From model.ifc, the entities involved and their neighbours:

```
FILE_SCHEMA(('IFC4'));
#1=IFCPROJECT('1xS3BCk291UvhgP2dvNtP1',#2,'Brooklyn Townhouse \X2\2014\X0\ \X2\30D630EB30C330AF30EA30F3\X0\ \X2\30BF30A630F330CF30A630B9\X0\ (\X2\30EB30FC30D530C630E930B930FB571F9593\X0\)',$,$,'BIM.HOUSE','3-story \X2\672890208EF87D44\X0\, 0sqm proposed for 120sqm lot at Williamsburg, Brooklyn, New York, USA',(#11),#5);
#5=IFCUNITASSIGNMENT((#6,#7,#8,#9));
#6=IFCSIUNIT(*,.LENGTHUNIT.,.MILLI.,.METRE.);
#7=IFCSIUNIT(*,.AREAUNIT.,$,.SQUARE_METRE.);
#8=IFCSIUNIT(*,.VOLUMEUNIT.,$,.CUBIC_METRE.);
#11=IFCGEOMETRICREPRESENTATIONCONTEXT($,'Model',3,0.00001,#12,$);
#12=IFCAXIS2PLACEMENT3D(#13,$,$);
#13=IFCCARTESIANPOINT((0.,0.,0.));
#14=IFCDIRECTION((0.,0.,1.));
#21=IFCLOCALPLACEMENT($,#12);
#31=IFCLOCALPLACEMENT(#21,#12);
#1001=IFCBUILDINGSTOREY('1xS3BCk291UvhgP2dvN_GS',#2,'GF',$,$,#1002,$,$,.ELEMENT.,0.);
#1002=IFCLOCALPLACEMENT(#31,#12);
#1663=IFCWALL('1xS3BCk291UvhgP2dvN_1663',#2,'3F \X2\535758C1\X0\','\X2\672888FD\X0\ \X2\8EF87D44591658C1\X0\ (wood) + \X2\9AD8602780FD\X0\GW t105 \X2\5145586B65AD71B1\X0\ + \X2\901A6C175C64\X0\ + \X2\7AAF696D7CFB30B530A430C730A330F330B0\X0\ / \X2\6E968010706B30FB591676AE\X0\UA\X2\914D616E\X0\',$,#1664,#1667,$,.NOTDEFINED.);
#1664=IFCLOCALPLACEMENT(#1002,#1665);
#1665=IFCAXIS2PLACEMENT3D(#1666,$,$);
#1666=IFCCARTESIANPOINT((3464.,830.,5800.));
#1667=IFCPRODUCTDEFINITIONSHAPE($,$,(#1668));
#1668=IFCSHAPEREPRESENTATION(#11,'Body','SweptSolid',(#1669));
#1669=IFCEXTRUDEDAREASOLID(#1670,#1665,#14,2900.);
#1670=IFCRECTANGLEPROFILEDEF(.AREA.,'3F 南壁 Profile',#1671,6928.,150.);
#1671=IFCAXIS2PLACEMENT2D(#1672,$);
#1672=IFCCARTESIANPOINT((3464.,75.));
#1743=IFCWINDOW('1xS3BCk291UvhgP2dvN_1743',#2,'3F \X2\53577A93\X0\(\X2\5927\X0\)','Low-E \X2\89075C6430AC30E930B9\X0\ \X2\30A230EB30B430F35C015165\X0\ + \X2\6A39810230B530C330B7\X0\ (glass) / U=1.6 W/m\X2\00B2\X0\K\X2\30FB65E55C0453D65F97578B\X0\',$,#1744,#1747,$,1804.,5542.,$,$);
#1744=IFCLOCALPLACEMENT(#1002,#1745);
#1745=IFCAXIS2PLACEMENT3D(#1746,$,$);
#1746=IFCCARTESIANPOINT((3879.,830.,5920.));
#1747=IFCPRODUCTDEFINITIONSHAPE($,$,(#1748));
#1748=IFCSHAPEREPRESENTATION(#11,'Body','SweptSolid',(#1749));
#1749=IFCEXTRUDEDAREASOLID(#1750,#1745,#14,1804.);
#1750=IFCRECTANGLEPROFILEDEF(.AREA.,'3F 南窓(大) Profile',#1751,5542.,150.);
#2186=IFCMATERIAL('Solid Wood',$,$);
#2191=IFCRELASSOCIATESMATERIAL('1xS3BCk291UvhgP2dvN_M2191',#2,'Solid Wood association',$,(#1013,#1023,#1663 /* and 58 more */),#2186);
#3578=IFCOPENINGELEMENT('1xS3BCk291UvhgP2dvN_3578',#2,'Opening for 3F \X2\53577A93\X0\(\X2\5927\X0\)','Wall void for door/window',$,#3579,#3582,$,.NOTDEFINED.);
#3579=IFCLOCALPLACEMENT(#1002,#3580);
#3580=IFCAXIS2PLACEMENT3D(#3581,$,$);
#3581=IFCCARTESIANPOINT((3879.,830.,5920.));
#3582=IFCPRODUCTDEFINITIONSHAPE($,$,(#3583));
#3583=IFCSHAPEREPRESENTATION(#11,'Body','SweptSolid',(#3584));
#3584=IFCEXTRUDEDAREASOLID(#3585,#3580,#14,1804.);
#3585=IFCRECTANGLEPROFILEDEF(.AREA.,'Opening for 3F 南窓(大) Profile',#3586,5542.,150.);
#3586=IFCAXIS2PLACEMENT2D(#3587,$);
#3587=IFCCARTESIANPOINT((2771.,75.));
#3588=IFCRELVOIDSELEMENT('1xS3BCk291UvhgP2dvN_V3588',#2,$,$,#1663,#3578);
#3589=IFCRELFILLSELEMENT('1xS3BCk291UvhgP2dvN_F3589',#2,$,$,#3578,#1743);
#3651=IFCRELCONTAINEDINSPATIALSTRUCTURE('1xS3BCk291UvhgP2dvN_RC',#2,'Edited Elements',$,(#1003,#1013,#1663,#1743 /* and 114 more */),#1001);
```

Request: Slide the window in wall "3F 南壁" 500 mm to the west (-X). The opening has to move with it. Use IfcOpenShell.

```python
import ifcopenshell
import ifcopenshell.api.geometry
import ifcopenshell.util.placement
import ifcopenshell.util.unit

model = ifcopenshell.open("model.ifc")
unit_scale = ifcopenshell.util.unit.calculate_unit_scale(model)

window = model.by_id(1743)
opening = window.FillsVoids[0].RelatingOpeningElement
wall = opening.VoidsElements[0].RelatingBuildingElement

wall_matrix = ifcopenshell.util.placement.get_local_placement(wall.ObjectPlacement)
shift = wall_matrix[:3, 0] * -0.5 / unit_scale
before = ifcopenshell.util.placement.get_local_placement(window.ObjectPlacement)[:3, 3].copy()

# The window is not placed relative to its opening, so move both.
for product in (opening, window):
    matrix = ifcopenshell.util.placement.get_local_placement(product.ObjectPlacement)
    matrix[:3, 3] += shift
    ifcopenshell.api.geometry.edit_object_placement(model, product=product, matrix=matrix, is_si=False)

after = ifcopenshell.util.placement.get_local_placement(window.ObjectPlacement)[:3, 3]
print("window moved by", (after - before).round(3) + 0.0)

model.write("model_v2.ifc")
```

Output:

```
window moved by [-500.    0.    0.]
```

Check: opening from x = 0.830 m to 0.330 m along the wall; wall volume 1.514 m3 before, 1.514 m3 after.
